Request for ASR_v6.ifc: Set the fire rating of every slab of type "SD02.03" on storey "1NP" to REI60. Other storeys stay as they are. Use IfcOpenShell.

First a look at what the model holds.

```python
import ifcopenshell
import ifcopenshell.util.element

model = ifcopenshell.open("ASR_v6.ifc")
print(model.schema)
storey = next(s for s in model.by_type("IfcBuildingStorey") if s.Name == "1NP")
slabs = [e for e in ifcopenshell.util.element.get_decomposition(storey) if e.is_a("IfcSlab")]
seen = {}
for e in slabs:
    element_type = ifcopenshell.util.element.get_type(e)
    key = (element_type.Name if element_type != e and element_type else None, ifcopenshell.util.element.get_pset(e, "Pset_SlabCommon", "FireRating"))
    seen[key] = seen.get(key, 0) + 1
for (name, value), count in sorted(seen.items(), key=str):
    print(count, "x", name, "|", value)
```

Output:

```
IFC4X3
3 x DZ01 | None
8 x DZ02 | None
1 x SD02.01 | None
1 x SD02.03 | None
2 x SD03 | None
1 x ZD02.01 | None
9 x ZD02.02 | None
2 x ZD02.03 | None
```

```python
import ifcopenshell
import ifcopenshell.api.pset
import ifcopenshell.util.element

model = ifcopenshell.open("ASR_v6.ifc")

storey = next(s for s in model.by_type("IfcBuildingStorey") if s.Name == "1NP")
slabs = [e for e in ifcopenshell.util.element.get_decomposition(storey) if e.is_a("IfcSlab")]

count = 0
for e in slabs:
    element_type = ifcopenshell.util.element.get_type(e)
    if element_type in (None, e) or element_type.Name != "SD02.03":
        continue
    # add_pset returns the element's existing set when there is one.
    pset = ifcopenshell.api.pset.add_pset(model, product=e, name="Pset_SlabCommon")
    ifcopenshell.api.pset.edit_pset(model, pset=pset, properties={"FireRating": "REI60"})
    count += 1

print(count, "slabs updated")

model.write("ASR_v6-out.ifc")
```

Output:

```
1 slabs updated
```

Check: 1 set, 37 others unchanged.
